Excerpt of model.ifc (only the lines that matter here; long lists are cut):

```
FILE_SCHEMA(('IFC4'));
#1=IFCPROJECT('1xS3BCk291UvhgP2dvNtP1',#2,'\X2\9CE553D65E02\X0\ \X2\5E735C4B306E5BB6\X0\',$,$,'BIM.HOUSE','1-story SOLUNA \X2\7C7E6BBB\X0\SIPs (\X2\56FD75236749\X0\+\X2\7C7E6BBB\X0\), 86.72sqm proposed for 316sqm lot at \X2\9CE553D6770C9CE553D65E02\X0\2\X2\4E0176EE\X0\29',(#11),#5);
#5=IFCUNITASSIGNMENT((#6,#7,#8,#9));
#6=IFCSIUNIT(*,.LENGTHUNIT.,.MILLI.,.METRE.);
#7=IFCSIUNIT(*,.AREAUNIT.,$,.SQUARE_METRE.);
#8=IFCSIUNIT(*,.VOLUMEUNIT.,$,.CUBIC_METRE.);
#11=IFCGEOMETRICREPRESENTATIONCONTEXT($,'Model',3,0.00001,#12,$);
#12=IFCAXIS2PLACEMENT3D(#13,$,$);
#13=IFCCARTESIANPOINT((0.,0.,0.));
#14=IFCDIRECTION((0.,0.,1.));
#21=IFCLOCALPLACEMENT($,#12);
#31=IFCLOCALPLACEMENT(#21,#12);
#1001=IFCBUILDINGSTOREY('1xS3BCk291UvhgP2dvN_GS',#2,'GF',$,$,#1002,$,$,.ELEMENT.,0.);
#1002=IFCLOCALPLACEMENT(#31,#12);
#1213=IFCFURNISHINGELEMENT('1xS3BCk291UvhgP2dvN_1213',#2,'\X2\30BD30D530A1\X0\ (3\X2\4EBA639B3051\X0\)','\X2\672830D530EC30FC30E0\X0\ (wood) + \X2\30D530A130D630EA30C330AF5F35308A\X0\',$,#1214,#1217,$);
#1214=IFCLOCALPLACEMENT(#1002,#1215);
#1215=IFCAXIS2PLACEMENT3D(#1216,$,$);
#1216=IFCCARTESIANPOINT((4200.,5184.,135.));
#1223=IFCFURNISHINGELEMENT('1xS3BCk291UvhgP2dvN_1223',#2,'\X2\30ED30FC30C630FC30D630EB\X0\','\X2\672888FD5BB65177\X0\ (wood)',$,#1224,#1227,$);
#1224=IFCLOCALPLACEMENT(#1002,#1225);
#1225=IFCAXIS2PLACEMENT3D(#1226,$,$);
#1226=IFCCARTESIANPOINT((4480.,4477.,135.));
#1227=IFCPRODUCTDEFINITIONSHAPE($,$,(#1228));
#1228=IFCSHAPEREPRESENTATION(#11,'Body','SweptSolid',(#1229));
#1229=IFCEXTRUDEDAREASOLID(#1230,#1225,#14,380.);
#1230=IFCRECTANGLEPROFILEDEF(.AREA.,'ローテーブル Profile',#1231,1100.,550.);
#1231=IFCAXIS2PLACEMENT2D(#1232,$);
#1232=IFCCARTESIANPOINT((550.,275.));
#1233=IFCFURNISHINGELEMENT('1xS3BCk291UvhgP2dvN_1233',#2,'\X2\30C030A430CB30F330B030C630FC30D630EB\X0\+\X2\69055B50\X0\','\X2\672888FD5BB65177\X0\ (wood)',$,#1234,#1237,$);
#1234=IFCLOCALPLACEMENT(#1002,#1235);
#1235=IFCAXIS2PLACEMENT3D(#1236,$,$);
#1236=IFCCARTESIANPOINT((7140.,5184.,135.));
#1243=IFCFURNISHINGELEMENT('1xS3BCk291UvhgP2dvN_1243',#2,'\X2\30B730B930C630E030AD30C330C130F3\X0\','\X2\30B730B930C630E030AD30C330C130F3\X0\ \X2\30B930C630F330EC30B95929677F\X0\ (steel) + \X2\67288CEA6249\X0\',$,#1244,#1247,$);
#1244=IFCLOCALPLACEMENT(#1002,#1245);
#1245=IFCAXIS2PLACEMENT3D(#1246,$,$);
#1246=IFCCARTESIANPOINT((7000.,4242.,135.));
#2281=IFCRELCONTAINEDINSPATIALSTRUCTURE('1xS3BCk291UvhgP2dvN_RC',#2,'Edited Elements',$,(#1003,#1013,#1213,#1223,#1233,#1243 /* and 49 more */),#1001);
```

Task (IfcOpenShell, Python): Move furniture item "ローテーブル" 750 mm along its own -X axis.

```python
import ifcopenshell
import ifcopenshell.api.geometry
import ifcopenshell.util.placement
import ifcopenshell.util.unit

model = ifcopenshell.open("model.ifc")
unit_scale = ifcopenshell.util.unit.calculate_unit_scale(model)

item = model.by_guid("1xS3BCk291UvhgP2dvN_1223")
matrix = ifcopenshell.util.placement.get_local_placement(item.ObjectPlacement)
matrix[:3, 3] -= matrix[:3, 0] * 0.75 / unit_scale
ifcopenshell.api.geometry.edit_object_placement(model, product=item, matrix=matrix, is_si=False)

print(ifcopenshell.util.placement.get_local_placement(item.ObjectPlacement).round(3) + 0.0)

model.write("model_rev.ifc")
```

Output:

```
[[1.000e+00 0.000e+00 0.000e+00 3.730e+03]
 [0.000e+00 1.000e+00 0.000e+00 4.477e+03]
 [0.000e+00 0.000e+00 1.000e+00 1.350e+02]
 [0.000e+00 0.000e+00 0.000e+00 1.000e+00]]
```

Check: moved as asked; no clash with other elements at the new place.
